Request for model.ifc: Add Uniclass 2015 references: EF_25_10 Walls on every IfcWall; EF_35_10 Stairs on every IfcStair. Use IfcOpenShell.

First a look at what the model holds.

```python
import ifcopenshell

model = ifcopenshell.open("model.ifc")
print(model.schema)
print("classifications:", [c.Name for c in model.by_type("IfcClassification")])
for ifc_class in ("IfcDoor", "IfcRoof", "IfcStair", "IfcWall", "IfcWindow"):
    print(ifc_class, len(model.by_type(ifc_class)))
```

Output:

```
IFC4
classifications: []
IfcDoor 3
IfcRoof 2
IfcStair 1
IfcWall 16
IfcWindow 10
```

```python
import ifcopenshell
import ifcopenshell.api.classification

model = ifcopenshell.open("model.ifc")

system = ifcopenshell.api.classification.add_classification(model, classification="Uniclass 2015")

codes = {
    "IfcWall": ("EF_25_10", "Walls"),
    "IfcStair": ("EF_35_10", "Stairs"),
}
for ifc_class, (code, name) in codes.items():
    products = model.by_type(ifc_class)
    ifcopenshell.api.classification.add_reference(
        model, products=products, classification=system, identification=code, name=name
    )
    print(code, len(products))

model.write("model_v2.ifc")
```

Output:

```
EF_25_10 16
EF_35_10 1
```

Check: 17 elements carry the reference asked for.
